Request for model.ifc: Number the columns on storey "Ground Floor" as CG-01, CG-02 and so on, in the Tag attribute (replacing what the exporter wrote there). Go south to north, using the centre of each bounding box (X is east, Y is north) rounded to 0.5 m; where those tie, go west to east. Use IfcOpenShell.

First a look at what the model holds.

```python
import ifcopenshell
import ifcopenshell.util.element
import ifcopenshell.util.placement

model = ifcopenshell.open("model.ifc")
print(model.schema)
storey = next(s for s in model.by_type("IfcBuildingStorey") if s.Name == "Ground Floor")
columns = [e for e in ifcopenshell.util.element.get_decomposition(storey) if e.is_a("IfcColumn")]
for e in sorted(columns, key=lambda e: e.id()):
    origin = ifcopenshell.util.placement.get_local_placement(e.ObjectPlacement)[:3, 3]
    print(e.id(), e.Tag, e.Name, origin.round(2) + 0.0, sep=" | ")
```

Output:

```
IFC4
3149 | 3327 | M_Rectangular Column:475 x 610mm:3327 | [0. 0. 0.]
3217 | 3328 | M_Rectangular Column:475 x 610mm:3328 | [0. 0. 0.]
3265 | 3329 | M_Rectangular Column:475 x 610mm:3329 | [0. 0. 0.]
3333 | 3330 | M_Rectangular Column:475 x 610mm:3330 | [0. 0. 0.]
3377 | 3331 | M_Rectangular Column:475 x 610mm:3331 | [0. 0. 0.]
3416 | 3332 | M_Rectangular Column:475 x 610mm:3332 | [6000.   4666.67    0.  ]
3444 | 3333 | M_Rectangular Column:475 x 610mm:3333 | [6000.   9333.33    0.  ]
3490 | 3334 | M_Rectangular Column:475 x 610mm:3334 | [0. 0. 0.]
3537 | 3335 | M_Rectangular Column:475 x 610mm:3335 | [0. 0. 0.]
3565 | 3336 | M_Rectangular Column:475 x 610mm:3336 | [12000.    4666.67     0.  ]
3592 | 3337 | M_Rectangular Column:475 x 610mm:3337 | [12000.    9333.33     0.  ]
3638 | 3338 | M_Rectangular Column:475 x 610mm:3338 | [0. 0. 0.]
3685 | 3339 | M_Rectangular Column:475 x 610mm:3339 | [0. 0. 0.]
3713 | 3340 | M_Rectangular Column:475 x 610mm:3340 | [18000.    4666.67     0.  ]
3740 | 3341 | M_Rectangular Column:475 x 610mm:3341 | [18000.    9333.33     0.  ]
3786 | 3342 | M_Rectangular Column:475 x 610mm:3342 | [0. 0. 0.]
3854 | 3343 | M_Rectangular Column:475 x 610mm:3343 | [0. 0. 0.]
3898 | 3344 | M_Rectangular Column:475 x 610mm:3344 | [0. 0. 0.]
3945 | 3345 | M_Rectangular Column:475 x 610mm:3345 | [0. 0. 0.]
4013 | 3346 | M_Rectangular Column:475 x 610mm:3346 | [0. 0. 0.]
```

```python
import ifcopenshell
import ifcopenshell.geom
import ifcopenshell.util.element
import ifcopenshell.util.shape

model = ifcopenshell.open("model.ifc")
settings = ifcopenshell.geom.settings()
settings.set("use-world-coords", True)


def centre(element):
    shape = ifcopenshell.geom.create_shape(settings, element)
    return ifcopenshell.util.shape.get_bbox_centroid(shape.geometry)


storey = next(s for s in model.by_type("IfcBuildingStorey") if s.Name == "Ground Floor")
columns = [e for e in ifcopenshell.util.element.get_decomposition(storey) if e.is_a("IfcColumn")]

# Insertion points can sit at a corner or the storey origin, so sort by the geometry (in metres).
centres = {e: centre(e) for e in columns}
columns.sort(key=lambda e: (round(centres[e][1] / 0.5), centres[e][0]))

for i, e in enumerate(columns, start=1):
    number = f"CG-{i:02d}"
    e.Tag = number
    print(e.id(), number)

model.write("model_edited.ifc")
```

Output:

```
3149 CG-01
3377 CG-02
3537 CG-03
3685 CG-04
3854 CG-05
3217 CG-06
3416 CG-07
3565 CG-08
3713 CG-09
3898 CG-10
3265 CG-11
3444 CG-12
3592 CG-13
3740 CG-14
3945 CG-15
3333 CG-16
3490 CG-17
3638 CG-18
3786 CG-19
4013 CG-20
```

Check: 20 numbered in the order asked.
